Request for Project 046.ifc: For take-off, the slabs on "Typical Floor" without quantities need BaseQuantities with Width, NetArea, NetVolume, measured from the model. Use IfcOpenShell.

First a look at what the model holds.

```python
import ifcopenshell
import ifcopenshell.util.element
import ifcopenshell.util.unit

model = ifcopenshell.open("Project 046.ifc")
print(model.schema)
for unit_type in ("LENGTHUNIT", "AREAUNIT", "VOLUMEUNIT"):
    print(unit_type, ifcopenshell.util.unit.calculate_unit_scale(model, unit_type))
storey = next(s for s in model.by_type("IfcBuildingStorey") if s.Name == "Typical Floor")
slabs = [e for e in ifcopenshell.util.element.get_decomposition(storey) if e.is_a("IfcSlab")]
for e in sorted(slabs, key=lambda e: e.id()):
    print(e.id(), e.is_a(), e.Name, list(ifcopenshell.util.element.get_psets(e, qtos_only=True)), sep=" | ")
```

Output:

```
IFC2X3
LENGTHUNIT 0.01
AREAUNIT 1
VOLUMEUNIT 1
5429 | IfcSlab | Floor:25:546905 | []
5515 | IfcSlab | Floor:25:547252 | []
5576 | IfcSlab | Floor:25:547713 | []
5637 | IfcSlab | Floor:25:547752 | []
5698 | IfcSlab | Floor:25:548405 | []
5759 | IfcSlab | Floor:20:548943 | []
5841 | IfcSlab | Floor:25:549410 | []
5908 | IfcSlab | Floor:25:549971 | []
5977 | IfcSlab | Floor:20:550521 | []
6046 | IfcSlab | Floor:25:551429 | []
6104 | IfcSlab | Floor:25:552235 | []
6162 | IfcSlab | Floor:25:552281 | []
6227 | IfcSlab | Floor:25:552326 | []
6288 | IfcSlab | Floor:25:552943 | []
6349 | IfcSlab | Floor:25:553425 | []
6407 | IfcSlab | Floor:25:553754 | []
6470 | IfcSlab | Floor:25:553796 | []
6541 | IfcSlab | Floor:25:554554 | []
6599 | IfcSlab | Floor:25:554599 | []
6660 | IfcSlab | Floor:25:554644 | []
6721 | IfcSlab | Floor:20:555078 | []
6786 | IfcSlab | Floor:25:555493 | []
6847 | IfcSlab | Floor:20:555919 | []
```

```python
import ifcopenshell
import ifcopenshell.api.pset
import ifcopenshell.geom
import ifcopenshell.util.element
import ifcopenshell.util.shape
import ifcopenshell.util.unit

model = ifcopenshell.open("Project 046.ifc")
unit_scale = ifcopenshell.util.unit.calculate_unit_scale(model)
area_scale = ifcopenshell.util.unit.calculate_unit_scale(model, "AREAUNIT")
volume_scale = ifcopenshell.util.unit.calculate_unit_scale(model, "VOLUMEUNIT")
settings = ifcopenshell.geom.settings()

storey = next(s for s in model.by_type("IfcBuildingStorey") if s.Name == "Typical Floor")
slabs = [e for e in ifcopenshell.util.element.get_decomposition(storey) if e.is_a("IfcSlab")]

for e in sorted(slabs, key=lambda e: e.id()):
    if ifcopenshell.util.element.get_psets(e, qtos_only=True, should_inherit=False):
        continue
    # Geometry comes back in metres, in the element's own axes.
    shape = ifcopenshell.geom.create_shape(settings, e)
    values = {
        "Width": ifcopenshell.util.shape.get_z(shape.geometry) / unit_scale,
        "NetArea": ifcopenshell.util.shape.get_footprint_area(shape.geometry) / area_scale,
        "NetVolume": ifcopenshell.util.shape.get_volume(shape.geometry) / volume_scale,
    }
    qto = ifcopenshell.api.pset.add_qto(model, product=e, name="BaseQuantities")
    ifcopenshell.api.pset.edit_qto(model, qto=qto, properties=values)
    print(e.id(), {k: round(v, 3) for k, v in values.items()})

model.write("Project 046_edited.ifc")
```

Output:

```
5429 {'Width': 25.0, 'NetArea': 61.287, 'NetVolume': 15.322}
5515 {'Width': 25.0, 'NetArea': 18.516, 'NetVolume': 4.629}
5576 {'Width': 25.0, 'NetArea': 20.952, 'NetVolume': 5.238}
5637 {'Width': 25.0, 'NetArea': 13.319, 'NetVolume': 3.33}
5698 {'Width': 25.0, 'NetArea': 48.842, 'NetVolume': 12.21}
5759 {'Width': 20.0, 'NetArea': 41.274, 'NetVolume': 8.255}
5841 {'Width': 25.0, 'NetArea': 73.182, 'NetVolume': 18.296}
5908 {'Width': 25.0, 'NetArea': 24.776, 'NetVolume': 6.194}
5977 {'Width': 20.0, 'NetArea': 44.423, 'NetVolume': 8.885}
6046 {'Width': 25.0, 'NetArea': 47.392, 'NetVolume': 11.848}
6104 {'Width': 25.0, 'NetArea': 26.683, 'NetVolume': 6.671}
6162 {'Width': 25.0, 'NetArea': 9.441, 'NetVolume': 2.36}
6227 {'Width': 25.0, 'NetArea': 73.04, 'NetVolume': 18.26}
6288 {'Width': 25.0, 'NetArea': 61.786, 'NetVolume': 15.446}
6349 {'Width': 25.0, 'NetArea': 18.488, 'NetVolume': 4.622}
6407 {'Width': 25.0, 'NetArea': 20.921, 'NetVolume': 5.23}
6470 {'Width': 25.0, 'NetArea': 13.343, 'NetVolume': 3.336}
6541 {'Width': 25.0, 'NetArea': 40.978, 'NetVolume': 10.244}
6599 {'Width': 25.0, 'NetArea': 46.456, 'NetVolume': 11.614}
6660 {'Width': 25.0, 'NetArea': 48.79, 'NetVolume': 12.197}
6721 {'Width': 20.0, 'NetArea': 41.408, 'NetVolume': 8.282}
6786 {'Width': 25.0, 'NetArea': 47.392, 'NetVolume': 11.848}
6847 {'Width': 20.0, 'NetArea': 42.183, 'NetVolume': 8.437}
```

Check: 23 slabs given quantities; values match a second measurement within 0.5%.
